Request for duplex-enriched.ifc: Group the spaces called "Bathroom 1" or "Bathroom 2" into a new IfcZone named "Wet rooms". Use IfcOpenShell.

First a look at what the model holds.

```python
import ifcopenshell

model = ifcopenshell.open("duplex-enriched.ifc")
print(model.schema)
seen = {}
for space in model.by_type("IfcSpace"):
    seen[space.LongName] = seen.get(space.LongName, 0) + 1
for name, count in sorted(seen.items(), key=str):
    print(count, "x", name)
print("zones:", [z.Name for z in model.by_type("IfcZone")][:20])
```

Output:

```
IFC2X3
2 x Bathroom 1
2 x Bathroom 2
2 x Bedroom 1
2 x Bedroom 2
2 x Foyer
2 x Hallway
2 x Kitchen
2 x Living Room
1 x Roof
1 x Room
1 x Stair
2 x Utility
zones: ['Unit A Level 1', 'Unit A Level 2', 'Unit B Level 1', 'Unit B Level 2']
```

```python
import ifcopenshell
import ifcopenshell.api.group
import ifcopenshell.api.root

model = ifcopenshell.open("duplex-enriched.ifc")

names = {"Bathroom 1", "Bathroom 2"}
spaces = [s for s in model.by_type("IfcSpace") if s.LongName in names]

zone = ifcopenshell.api.root.create_entity(model, ifc_class="IfcZone", name="Wet rooms")
ifcopenshell.api.group.assign_group(model, products=spaces, group=zone)
print(len(spaces), "spaces in", zone.Name)

model.write("duplex-enriched_rev.ifc")
```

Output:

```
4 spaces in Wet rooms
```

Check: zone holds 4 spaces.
